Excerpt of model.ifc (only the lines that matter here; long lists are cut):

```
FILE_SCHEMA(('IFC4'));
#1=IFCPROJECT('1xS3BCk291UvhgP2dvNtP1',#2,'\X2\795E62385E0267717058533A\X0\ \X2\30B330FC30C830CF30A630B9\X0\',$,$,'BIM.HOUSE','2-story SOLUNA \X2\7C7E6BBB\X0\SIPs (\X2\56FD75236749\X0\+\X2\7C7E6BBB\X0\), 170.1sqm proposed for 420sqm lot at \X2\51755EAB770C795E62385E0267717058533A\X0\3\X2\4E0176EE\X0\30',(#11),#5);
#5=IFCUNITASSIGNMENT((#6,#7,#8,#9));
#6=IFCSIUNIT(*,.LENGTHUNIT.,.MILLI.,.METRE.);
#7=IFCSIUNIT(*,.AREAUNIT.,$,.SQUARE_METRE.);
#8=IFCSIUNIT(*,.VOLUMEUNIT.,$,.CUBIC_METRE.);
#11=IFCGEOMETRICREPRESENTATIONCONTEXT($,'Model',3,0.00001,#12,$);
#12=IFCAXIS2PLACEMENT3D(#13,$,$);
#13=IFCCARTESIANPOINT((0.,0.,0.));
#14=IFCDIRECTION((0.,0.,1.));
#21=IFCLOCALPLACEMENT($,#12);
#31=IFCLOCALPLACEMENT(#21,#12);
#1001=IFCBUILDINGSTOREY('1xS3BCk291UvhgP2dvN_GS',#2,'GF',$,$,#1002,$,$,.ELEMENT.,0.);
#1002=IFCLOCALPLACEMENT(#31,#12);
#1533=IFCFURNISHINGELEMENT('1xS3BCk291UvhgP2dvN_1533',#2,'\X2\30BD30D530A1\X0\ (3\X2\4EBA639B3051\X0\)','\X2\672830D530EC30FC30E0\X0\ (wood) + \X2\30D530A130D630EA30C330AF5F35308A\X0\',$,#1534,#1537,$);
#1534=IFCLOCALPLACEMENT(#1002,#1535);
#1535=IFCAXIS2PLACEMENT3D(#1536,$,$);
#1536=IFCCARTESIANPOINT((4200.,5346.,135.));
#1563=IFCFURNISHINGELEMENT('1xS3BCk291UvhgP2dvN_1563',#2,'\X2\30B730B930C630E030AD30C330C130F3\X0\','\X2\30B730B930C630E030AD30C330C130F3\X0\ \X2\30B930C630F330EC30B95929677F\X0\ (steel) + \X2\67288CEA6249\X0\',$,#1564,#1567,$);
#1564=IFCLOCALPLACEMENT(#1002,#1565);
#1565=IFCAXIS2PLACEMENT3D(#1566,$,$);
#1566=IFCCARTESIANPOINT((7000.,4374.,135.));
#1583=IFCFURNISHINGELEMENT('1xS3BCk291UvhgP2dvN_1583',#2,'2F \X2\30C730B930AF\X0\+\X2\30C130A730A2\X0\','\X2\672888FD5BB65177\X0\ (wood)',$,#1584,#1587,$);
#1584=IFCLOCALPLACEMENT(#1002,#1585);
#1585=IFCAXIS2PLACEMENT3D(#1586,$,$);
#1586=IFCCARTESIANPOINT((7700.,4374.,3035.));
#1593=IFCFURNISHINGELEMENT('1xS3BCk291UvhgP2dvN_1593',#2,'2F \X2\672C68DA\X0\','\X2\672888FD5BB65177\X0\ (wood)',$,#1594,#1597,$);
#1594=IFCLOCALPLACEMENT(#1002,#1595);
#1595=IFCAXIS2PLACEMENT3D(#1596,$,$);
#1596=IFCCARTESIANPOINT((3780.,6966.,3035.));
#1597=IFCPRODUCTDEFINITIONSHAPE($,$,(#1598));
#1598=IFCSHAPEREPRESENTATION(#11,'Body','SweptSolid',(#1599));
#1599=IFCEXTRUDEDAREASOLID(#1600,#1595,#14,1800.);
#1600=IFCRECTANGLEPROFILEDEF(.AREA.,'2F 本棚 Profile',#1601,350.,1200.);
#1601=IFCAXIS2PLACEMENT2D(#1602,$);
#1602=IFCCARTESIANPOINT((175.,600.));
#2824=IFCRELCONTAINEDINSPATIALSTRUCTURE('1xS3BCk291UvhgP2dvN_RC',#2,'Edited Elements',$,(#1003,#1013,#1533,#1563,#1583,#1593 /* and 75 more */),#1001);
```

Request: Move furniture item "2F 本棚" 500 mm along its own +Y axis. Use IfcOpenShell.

```python
import ifcopenshell
import ifcopenshell.api.geometry
import ifcopenshell.util.placement

model = ifcopenshell.open("model.ifc")

item = model.by_guid("1xS3BCk291UvhgP2dvN_1593")
matrix = ifcopenshell.util.placement.get_local_placement(item.ObjectPlacement)
matrix[:3, 3] += matrix[:3, 1] * 500.0
ifcopenshell.api.geometry.edit_object_placement(model, product=item, matrix=matrix, is_si=False)

print(ifcopenshell.util.placement.get_local_placement(item.ObjectPlacement).round(3) + 0.0)

model.write("model-out.ifc")
```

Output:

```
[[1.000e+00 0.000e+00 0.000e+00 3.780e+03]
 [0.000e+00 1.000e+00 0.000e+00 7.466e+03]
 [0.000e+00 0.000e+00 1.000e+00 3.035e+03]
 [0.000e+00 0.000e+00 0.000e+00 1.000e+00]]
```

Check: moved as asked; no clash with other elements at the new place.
